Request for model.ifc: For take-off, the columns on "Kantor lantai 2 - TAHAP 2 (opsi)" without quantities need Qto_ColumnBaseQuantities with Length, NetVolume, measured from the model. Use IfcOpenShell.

First a look at what the model holds.

```python
import ifcopenshell
import ifcopenshell.util.element
import ifcopenshell.util.unit

model = ifcopenshell.open("model.ifc")
print(model.schema)
for unit_type in ("LENGTHUNIT", "AREAUNIT", "VOLUMEUNIT"):
    print(unit_type, ifcopenshell.util.unit.calculate_unit_scale(model, unit_type))
storey = next(s for s in model.by_type("IfcBuildingStorey") if s.Name == "Kantor lantai 2 - TAHAP 2 (opsi)")
columns = [e for e in ifcopenshell.util.element.get_decomposition(storey) if e.is_a("IfcColumn")]
for e in sorted(columns, key=lambda e: e.id()):
    print(e.id(), e.is_a(), e.Name, list(ifcopenshell.util.element.get_psets(e, qtos_only=True)), sep=" | ")
```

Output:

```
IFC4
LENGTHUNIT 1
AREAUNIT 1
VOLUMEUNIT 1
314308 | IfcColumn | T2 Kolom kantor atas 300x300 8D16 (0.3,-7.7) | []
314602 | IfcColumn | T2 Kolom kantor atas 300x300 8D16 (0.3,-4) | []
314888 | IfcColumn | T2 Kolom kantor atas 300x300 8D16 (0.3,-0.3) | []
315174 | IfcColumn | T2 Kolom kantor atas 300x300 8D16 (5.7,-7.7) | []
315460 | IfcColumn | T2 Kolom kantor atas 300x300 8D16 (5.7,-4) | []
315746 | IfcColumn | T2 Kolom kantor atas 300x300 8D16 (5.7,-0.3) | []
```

```python
import ifcopenshell
import ifcopenshell.api.pset
import ifcopenshell.geom
import ifcopenshell.util.element
import ifcopenshell.util.shape
import ifcopenshell.util.unit

model = ifcopenshell.open("model.ifc")
unit_scale = ifcopenshell.util.unit.calculate_unit_scale(model)
volume_scale = ifcopenshell.util.unit.calculate_unit_scale(model, "VOLUMEUNIT")
settings = ifcopenshell.geom.settings()

storey = next(s for s in model.by_type("IfcBuildingStorey") if s.Name == "Kantor lantai 2 - TAHAP 2 (opsi)")
columns = [e for e in ifcopenshell.util.element.get_decomposition(storey) if e.is_a("IfcColumn")]

for e in sorted(columns, key=lambda e: e.id()):
    if ifcopenshell.util.element.get_psets(e, qtos_only=True, should_inherit=False):
        continue
    # Geometry comes back in metres, in the element's own axes.
    shape = ifcopenshell.geom.create_shape(settings, e)
    values = {
        "Length": ifcopenshell.util.shape.get_z(shape.geometry) / unit_scale,
        "NetVolume": ifcopenshell.util.shape.get_volume(shape.geometry) / volume_scale,
    }
    qto = ifcopenshell.api.pset.add_qto(model, product=e, name="Qto_ColumnBaseQuantities")
    ifcopenshell.api.pset.edit_qto(model, qto=qto, properties=values)
    print(e.id(), {k: round(v, 3) for k, v in values.items()})

model.write("model-out.ifc")
```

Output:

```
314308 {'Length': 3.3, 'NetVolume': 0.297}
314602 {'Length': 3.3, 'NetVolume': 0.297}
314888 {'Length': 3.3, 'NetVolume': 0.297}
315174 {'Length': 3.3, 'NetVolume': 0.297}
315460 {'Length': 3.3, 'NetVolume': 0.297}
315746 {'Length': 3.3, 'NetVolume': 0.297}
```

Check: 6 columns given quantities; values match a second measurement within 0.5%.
